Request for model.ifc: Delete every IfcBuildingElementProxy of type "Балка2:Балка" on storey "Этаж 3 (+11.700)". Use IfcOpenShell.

First a look at what the model holds.

```python
import ifcopenshell
import ifcopenshell.util.element

model = ifcopenshell.open("model.ifc")
print(model.schema)
storey = next(s for s in model.by_type("IfcBuildingStorey") if s.Name == "Этаж 3 (+11.700)")
proxies = [e for e in ifcopenshell.util.element.get_decomposition(storey) if e.is_a("IfcBuildingElementProxy")]
seen = {}
for e in proxies:
    element_type = ifcopenshell.util.element.get_type(e)
    name = element_type.Name if element_type not in (None, e) else None
    seen[name] = seen.get(name, 0) + 1
for name, count in sorted(seen.items(), key=str):
    print(count, "x", name)
```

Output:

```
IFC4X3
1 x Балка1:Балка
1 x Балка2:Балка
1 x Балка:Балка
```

```python
import ifcopenshell
import ifcopenshell.api.root
import ifcopenshell.util.element

model = ifcopenshell.open("model.ifc")

storey = next(s for s in model.by_type("IfcBuildingStorey") if s.Name == "Этаж 3 (+11.700)")
proxies = [e for e in ifcopenshell.util.element.get_decomposition(storey) if e.is_a("IfcBuildingElementProxy")]
targets = [e for e in proxies if (t := ifcopenshell.util.element.get_type(e)) not in (None, e) and t.Name == "Балка2:Балка"]

for e in targets:
    ifcopenshell.api.root.remove_product(model, product=e)
print(len(targets), "removed")

model.write("model_rev.ifc")
```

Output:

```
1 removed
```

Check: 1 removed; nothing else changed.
